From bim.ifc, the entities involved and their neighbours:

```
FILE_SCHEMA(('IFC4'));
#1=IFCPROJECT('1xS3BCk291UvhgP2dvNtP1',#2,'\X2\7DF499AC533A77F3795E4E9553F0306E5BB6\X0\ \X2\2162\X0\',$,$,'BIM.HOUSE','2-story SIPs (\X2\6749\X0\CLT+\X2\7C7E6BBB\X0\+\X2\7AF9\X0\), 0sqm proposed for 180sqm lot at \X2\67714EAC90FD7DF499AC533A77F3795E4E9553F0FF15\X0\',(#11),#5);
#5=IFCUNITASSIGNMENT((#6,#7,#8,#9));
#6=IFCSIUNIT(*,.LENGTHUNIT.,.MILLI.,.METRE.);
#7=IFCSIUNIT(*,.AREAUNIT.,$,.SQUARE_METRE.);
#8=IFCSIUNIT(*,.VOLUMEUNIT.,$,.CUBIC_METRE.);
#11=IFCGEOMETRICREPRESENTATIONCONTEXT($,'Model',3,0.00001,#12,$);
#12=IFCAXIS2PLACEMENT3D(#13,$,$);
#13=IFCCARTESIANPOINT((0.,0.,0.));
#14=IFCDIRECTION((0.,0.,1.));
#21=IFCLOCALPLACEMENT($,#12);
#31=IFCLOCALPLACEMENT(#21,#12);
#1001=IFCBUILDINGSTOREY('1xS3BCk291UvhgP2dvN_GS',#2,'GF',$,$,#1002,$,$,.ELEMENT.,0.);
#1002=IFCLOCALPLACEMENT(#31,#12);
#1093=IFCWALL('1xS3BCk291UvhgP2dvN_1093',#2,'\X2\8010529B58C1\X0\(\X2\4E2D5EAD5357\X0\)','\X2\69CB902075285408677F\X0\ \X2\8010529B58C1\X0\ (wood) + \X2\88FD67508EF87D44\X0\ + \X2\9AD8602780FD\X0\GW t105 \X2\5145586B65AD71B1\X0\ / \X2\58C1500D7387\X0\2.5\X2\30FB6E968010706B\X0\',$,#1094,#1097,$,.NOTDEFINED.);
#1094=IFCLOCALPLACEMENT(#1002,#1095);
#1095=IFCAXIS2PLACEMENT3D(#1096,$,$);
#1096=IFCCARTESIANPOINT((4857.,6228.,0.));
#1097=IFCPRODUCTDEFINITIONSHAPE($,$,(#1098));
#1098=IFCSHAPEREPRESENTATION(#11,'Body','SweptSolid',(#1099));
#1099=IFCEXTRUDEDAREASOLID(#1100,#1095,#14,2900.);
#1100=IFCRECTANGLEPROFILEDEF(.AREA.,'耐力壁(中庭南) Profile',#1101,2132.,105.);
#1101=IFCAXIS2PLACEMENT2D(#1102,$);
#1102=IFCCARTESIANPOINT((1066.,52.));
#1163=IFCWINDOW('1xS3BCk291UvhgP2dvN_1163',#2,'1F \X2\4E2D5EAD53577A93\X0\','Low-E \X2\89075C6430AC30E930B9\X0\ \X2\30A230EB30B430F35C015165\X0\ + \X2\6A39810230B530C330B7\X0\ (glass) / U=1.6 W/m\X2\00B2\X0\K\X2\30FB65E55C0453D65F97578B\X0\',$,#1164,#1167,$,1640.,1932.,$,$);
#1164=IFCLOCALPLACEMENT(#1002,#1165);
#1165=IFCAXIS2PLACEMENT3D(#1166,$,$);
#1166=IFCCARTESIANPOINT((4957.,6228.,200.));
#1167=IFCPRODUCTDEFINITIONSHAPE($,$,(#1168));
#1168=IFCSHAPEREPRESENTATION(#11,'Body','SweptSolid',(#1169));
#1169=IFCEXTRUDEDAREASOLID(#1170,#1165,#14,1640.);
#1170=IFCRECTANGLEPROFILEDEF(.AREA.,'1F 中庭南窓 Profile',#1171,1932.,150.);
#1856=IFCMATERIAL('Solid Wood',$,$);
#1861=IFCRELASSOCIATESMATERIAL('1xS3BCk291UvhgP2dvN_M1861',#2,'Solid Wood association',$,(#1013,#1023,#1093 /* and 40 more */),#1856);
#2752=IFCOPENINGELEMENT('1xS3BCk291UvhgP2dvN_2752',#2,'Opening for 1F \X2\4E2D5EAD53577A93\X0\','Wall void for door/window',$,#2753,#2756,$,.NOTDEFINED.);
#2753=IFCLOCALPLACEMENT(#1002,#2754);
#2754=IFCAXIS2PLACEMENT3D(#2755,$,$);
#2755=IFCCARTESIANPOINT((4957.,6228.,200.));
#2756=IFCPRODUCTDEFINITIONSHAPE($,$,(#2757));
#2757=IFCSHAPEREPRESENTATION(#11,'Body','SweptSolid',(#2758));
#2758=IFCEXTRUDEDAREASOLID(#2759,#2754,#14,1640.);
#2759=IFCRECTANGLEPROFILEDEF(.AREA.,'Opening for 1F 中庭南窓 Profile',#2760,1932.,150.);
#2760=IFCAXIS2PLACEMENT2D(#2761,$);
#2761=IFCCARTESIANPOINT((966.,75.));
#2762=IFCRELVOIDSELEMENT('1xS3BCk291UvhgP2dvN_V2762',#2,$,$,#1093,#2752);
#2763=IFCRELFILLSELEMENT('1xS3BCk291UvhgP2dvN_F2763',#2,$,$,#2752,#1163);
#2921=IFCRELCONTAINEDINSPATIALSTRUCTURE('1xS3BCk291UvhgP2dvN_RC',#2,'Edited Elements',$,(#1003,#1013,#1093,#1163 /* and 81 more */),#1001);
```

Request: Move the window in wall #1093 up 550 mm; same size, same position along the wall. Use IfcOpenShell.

```python
import numpy as np
import ifcopenshell
import ifcopenshell.api.geometry
import ifcopenshell.util.placement
import ifcopenshell.util.unit

model = ifcopenshell.open("bim.ifc")
unit_scale = ifcopenshell.util.unit.calculate_unit_scale(model)

window = model.by_id(1163)
opening = window.FillsVoids[0].RelatingOpeningElement
dz = 0.55 / unit_scale

shift = np.array([0.0, 0.0, dz])
# The window is not placed relative to its opening, so move both.
for product in (opening, window):
    matrix = ifcopenshell.util.placement.get_local_placement(product.ObjectPlacement)
    matrix[:3, 3] += shift
    ifcopenshell.api.geometry.edit_object_placement(model, product=product, matrix=matrix, is_si=False)

print(f"moved by {dz * unit_scale:+.3f} m")

model.write("bim_v2.ifc")
```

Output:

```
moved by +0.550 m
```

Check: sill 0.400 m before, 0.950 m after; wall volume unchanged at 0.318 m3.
